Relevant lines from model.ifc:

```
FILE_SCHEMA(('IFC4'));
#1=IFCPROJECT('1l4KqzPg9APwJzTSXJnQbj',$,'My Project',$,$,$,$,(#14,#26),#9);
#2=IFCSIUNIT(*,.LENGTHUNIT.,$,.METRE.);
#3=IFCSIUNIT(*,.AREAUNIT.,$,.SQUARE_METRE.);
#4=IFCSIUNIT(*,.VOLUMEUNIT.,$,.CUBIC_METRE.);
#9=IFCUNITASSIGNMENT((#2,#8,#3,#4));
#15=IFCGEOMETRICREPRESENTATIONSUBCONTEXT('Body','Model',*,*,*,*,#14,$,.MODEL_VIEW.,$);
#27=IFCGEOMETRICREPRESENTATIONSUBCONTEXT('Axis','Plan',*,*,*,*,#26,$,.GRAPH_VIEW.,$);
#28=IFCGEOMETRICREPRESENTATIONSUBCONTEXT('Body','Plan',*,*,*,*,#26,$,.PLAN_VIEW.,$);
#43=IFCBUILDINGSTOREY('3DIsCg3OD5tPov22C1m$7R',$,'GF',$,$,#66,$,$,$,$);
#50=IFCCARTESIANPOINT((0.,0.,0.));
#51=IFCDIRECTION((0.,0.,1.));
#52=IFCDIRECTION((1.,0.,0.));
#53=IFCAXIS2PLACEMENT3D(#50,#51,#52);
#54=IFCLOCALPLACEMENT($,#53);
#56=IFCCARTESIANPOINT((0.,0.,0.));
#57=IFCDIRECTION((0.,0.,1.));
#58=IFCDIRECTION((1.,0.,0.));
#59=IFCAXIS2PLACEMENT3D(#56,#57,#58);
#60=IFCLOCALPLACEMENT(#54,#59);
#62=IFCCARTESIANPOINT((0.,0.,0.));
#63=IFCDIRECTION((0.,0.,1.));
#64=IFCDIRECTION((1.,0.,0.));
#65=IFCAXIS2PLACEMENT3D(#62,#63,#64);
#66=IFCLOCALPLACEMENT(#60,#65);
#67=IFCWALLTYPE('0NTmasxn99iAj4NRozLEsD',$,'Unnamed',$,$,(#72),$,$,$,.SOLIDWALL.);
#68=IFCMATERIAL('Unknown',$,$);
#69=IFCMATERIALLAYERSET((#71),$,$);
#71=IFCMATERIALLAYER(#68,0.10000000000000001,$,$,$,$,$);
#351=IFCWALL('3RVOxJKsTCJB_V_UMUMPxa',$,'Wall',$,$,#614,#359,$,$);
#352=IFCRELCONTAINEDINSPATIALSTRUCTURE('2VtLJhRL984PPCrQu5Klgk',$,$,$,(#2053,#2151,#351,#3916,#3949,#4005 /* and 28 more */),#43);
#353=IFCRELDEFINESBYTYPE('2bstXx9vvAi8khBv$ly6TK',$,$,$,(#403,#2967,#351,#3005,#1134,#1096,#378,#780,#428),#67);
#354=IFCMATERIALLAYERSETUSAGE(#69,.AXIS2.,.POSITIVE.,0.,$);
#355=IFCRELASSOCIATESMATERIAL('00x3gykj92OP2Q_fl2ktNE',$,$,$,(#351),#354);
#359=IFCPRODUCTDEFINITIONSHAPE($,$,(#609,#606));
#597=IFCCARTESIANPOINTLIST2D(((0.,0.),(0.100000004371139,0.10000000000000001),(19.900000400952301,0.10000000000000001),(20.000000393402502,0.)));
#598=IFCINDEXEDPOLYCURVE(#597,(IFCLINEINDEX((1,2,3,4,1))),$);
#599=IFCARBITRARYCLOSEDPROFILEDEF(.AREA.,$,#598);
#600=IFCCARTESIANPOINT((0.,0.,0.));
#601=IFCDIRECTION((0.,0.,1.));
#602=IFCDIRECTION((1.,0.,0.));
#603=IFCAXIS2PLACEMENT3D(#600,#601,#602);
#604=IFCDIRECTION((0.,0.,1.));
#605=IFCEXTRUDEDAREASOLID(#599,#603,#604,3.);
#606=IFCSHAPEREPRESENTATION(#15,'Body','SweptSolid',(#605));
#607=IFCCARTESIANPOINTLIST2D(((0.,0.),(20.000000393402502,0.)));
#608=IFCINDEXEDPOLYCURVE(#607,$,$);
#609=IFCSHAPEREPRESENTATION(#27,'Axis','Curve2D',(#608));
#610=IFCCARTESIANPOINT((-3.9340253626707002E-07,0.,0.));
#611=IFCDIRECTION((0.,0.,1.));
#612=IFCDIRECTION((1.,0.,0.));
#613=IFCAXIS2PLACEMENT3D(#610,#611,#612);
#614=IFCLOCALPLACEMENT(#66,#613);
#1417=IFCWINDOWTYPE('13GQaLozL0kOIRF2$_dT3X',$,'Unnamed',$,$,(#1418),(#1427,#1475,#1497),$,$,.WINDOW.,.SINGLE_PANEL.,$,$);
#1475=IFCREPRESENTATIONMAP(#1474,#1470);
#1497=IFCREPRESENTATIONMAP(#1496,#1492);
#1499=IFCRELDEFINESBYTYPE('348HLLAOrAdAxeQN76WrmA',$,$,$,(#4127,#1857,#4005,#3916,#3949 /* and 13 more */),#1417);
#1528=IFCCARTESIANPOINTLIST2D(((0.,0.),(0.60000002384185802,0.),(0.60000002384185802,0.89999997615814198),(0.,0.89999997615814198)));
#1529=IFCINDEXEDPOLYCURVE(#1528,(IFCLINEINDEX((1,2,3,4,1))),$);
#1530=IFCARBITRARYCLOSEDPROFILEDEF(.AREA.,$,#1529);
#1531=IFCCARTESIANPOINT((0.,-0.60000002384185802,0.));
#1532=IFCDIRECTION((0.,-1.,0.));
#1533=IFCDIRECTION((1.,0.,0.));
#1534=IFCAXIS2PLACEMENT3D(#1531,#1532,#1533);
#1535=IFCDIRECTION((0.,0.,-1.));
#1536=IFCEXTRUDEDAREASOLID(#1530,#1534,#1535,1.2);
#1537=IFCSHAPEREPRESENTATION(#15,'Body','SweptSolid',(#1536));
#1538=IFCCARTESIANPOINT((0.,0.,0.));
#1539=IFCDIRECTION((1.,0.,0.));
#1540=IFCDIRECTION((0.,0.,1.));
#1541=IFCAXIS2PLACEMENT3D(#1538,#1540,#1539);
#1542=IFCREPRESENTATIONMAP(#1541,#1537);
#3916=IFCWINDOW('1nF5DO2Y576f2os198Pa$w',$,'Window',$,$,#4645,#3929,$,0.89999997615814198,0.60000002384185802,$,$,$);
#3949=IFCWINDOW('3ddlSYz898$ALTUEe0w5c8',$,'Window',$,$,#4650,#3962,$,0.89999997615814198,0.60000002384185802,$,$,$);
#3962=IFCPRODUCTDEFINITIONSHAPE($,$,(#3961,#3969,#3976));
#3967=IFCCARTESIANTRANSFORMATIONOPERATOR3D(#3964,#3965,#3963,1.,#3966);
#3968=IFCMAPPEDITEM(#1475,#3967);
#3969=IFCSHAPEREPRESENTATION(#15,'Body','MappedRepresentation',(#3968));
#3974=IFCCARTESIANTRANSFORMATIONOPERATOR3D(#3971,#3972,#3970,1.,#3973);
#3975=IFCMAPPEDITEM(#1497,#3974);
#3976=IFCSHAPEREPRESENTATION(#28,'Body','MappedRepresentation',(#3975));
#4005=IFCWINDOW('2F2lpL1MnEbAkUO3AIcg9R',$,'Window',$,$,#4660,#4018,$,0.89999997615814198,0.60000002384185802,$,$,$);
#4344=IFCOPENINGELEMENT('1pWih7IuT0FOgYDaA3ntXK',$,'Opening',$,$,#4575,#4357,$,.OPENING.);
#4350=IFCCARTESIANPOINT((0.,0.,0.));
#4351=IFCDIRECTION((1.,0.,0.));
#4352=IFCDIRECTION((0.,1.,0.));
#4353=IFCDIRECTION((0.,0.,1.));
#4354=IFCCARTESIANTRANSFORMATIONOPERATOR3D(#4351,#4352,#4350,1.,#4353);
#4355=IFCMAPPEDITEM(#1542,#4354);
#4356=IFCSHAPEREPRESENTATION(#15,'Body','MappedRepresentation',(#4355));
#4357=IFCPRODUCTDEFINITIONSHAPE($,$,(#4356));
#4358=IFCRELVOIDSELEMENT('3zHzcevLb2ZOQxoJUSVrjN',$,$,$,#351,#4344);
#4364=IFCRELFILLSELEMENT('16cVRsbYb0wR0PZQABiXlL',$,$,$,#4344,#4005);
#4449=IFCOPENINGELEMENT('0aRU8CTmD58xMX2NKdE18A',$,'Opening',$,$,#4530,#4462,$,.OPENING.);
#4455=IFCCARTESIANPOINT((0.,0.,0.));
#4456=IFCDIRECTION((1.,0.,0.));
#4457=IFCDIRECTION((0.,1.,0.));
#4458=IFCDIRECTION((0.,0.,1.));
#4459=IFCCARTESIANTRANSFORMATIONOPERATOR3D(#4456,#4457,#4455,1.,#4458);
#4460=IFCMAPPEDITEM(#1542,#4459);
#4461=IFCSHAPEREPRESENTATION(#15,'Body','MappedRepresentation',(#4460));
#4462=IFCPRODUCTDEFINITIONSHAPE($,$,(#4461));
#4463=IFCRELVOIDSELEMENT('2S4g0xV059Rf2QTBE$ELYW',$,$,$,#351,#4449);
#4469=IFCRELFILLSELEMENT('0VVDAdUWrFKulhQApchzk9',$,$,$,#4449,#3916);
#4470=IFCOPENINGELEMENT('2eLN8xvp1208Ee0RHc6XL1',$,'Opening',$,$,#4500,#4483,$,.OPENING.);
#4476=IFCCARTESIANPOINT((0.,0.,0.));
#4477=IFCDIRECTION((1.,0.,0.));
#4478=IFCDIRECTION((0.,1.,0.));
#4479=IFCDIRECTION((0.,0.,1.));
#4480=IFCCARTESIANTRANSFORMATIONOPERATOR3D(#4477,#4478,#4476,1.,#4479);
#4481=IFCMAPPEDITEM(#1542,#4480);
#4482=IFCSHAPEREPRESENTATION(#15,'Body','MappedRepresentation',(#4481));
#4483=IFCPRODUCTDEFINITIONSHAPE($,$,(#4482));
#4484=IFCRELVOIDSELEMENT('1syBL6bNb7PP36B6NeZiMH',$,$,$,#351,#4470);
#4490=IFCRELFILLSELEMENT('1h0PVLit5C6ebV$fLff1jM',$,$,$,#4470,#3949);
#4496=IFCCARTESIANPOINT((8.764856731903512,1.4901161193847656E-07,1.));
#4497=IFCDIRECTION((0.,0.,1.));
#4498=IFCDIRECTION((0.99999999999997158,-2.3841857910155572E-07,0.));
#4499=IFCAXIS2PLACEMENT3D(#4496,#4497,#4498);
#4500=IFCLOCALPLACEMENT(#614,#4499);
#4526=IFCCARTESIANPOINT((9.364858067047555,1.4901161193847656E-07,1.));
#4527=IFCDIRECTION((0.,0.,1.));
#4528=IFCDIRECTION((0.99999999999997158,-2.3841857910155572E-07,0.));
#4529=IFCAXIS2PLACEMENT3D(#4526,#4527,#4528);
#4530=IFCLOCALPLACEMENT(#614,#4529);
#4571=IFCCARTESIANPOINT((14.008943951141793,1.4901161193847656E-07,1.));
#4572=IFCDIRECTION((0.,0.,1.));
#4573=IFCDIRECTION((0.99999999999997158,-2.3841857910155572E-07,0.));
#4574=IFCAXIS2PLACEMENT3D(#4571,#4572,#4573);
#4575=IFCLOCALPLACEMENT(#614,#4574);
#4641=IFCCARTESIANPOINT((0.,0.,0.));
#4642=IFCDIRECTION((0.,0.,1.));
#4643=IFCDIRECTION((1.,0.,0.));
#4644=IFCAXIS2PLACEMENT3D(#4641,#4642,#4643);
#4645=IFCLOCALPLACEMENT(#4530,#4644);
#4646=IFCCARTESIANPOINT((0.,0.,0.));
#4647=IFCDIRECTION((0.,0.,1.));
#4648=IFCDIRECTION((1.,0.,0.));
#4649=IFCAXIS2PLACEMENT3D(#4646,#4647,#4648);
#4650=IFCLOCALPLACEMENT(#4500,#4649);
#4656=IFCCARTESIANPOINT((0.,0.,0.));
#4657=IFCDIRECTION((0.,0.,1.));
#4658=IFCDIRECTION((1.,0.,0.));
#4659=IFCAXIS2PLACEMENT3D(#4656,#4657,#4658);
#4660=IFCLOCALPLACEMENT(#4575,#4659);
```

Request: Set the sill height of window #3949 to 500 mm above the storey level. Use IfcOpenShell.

```python
import numpy as np
import ifcopenshell
import ifcopenshell.api.geometry
import ifcopenshell.geom
import ifcopenshell.util.element
import ifcopenshell.util.placement
import ifcopenshell.util.shape
import ifcopenshell.util.unit

model = ifcopenshell.open("model.ifc")
unit_scale = ifcopenshell.util.unit.calculate_unit_scale(model)

window = model.by_id(3949)
opening = window.FillsVoids[0].RelatingOpeningElement
storey = ifcopenshell.util.element.get_container(window, ifc_class="IfcBuildingStorey")
level = ifcopenshell.util.placement.get_local_placement(storey.ObjectPlacement)[2, 3]

# The opening's origin need not be at the sill, so measure its lowest point.
shape = ifcopenshell.geom.create_shape(ifcopenshell.geom.settings(), opening)
bottom = ifcopenshell.util.shape.get_shape_bottom_elevation(shape, shape.geometry) / unit_scale
dz = level + 0.5 / unit_scale - bottom

shift = np.array([0.0, 0.0, dz])
# The window is placed relative to its opening, so it follows when the opening moves.
matrix = ifcopenshell.util.placement.get_local_placement(opening.ObjectPlacement)
matrix[:3, 3] += shift
ifcopenshell.api.geometry.edit_object_placement(
    model, product=opening, matrix=matrix, is_si=False, should_transform_children=True
)

print(f"moved by {dz * unit_scale:+.3f} m")

model.write("model_updated.ifc")
```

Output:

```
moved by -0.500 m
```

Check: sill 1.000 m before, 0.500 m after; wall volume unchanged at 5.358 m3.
